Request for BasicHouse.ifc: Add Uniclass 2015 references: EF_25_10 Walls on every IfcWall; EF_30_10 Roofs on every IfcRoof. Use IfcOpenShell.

First a look at what the model holds.

```python
import ifcopenshell

model = ifcopenshell.open("BasicHouse.ifc")
print(model.schema)
print("classifications:", [c.Name for c in model.by_type("IfcClassification")])
for ifc_class in ("IfcDoor", "IfcRoof", "IfcStair", "IfcWall", "IfcWindow"):
    print(ifc_class, len(model.by_type(ifc_class)))
```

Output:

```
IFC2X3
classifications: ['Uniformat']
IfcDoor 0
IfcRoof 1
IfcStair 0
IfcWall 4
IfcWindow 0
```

```python
import ifcopenshell
import ifcopenshell.api.classification

model = ifcopenshell.open("BasicHouse.ifc")

# IFC2X3 requires Source and Edition and has no link from the project to the system.
system = model.create_entity("IfcClassification", Source="NBS", Edition="2015", Name="Uniclass 2015")

codes = {
    "IfcWall": ("EF_25_10", "Walls"),
    "IfcRoof": ("EF_30_10", "Roofs"),
}
for ifc_class, (code, name) in codes.items():
    products = model.by_type(ifc_class)
    ifcopenshell.api.classification.add_reference(
        model, products=products, classification=system, identification=code, name=name
    )
    print(code, len(products))

model.write("BasicHouse_updated.ifc")
```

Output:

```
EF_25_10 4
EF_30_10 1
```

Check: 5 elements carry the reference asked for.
